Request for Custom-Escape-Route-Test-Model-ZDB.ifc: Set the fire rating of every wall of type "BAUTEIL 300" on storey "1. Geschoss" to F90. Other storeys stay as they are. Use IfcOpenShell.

First a look at what the model holds.

```python
import ifcopenshell
import ifcopenshell.util.element

model = ifcopenshell.open("Custom-Escape-Route-Test-Model-ZDB.ifc")
print(model.schema)
storey = next(s for s in model.by_type("IfcBuildingStorey") if s.Name == "1. Geschoss")
walls = [e for e in ifcopenshell.util.element.get_decomposition(storey) if e.is_a("IfcWall")]
seen = {}
for e in walls:
    element_type = ifcopenshell.util.element.get_type(e)
    key = (element_type.Name if element_type != e and element_type else None, ifcopenshell.util.element.get_pset(e, "Pset_WallCommon", "FireRating"))
    seen[key] = seen.get(key, 0) + 1
for (name, value), count in sorted(seen.items(), key=str):
    print(count, "x", name, "|", value)
```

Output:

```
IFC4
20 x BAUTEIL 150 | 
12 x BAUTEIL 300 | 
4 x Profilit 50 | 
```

```python
import ifcopenshell
import ifcopenshell.api.pset
import ifcopenshell.util.element

model = ifcopenshell.open("Custom-Escape-Route-Test-Model-ZDB.ifc")

storey = next(s for s in model.by_type("IfcBuildingStorey") if s.Name == "1. Geschoss")
walls = [e for e in ifcopenshell.util.element.get_decomposition(storey) if e.is_a("IfcWall")]

count = 0
for e in walls:
    element_type = ifcopenshell.util.element.get_type(e)
    if element_type in (None, e) or element_type.Name != "BAUTEIL 300":
        continue
    # add_pset returns the element's existing set when there is one.
    pset = ifcopenshell.api.pset.add_pset(model, product=e, name="Pset_WallCommon")
    ifcopenshell.api.pset.edit_pset(model, pset=pset, properties={"FireRating": "F90"})
    count += 1

print(count, "walls updated")

model.write("Custom-Escape-Route-Test-Model-ZDB_rev.ifc")
```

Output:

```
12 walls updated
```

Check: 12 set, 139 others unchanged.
